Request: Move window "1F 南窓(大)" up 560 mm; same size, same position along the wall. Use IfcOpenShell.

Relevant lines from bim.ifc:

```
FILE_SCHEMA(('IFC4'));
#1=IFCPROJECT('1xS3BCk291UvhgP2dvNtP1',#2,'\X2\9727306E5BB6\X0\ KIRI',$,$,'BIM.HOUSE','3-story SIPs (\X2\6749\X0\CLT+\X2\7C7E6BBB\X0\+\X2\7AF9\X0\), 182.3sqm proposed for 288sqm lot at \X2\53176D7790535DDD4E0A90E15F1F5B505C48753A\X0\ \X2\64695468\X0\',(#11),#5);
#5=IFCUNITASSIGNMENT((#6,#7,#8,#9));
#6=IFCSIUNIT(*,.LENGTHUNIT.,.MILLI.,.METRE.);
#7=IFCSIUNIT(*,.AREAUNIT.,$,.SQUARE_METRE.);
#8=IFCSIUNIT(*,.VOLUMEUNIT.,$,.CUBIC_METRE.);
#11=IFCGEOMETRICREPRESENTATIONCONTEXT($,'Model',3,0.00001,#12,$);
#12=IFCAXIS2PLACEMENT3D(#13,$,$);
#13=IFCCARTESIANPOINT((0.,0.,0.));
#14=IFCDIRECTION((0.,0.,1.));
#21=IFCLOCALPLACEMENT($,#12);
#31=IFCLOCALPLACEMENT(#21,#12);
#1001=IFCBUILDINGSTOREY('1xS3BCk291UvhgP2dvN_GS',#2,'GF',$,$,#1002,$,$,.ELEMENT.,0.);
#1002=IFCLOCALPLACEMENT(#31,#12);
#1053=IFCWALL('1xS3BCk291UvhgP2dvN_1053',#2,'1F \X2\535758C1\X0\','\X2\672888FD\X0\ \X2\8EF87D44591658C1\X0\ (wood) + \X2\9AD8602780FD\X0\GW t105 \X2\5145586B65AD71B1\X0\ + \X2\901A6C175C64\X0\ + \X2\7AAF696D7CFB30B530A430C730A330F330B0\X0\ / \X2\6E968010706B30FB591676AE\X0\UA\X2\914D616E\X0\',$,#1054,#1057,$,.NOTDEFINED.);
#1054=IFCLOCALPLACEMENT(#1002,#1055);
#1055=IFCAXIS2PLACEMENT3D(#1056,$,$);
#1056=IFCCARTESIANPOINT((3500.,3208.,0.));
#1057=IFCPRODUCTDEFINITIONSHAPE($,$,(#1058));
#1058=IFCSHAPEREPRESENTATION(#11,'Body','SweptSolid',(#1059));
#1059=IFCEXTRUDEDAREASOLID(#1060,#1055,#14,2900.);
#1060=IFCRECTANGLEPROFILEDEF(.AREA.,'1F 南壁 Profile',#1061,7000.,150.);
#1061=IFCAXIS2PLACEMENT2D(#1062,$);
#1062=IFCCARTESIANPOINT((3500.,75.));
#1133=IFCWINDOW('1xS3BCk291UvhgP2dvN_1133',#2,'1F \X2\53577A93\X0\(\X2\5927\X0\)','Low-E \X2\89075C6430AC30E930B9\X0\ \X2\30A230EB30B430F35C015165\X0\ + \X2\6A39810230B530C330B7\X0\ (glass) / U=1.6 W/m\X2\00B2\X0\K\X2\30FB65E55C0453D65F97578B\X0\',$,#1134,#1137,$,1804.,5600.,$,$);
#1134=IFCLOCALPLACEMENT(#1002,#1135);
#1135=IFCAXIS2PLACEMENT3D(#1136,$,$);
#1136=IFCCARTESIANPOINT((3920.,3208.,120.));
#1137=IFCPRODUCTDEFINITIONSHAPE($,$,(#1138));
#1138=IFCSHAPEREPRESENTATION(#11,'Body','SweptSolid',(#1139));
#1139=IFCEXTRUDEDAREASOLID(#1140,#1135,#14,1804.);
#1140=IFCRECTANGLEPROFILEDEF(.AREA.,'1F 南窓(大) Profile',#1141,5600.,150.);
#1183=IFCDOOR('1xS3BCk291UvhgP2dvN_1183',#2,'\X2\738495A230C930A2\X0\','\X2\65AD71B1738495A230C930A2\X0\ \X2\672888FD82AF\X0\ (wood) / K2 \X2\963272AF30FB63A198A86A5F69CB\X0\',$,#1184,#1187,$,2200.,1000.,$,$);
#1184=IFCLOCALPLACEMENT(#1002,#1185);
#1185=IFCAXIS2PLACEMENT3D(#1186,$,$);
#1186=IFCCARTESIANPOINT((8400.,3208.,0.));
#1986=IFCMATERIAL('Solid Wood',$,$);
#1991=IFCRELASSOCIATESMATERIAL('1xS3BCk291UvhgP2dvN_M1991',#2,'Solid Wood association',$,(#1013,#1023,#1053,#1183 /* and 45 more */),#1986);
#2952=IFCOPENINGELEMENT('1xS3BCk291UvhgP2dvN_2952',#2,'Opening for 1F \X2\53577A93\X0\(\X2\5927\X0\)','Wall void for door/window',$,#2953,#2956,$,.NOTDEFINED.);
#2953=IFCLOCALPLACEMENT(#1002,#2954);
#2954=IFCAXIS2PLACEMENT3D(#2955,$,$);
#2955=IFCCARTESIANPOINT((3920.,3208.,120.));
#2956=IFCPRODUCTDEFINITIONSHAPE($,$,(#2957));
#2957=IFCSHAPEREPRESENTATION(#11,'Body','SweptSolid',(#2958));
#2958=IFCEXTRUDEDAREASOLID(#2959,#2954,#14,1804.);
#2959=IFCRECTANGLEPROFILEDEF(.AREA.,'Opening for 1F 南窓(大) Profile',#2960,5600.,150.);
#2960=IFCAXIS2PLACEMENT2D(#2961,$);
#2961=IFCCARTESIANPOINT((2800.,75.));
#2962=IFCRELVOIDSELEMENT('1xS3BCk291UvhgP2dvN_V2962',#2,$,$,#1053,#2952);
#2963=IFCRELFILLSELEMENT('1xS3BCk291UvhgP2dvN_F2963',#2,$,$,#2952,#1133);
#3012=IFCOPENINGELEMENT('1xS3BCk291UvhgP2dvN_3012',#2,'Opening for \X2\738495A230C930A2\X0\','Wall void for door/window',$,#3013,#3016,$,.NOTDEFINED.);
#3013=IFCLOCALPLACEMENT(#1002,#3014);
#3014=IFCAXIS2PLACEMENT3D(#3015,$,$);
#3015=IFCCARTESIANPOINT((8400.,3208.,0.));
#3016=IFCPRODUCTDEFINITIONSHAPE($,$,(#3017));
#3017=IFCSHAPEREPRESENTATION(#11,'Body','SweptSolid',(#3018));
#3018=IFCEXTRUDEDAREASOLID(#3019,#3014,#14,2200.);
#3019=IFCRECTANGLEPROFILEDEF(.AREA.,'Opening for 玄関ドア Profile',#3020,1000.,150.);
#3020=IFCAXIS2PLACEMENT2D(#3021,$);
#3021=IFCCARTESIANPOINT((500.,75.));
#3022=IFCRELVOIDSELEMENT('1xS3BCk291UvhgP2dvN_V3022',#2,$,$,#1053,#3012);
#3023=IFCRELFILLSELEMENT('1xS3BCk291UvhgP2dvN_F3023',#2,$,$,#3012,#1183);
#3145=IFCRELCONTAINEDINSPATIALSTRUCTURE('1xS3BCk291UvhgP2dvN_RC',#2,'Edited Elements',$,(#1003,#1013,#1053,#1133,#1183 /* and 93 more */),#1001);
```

```python
import numpy as np
import ifcopenshell
import ifcopenshell.api.geometry
import ifcopenshell.util.placement
import ifcopenshell.util.unit

model = ifcopenshell.open("bim.ifc")
unit_scale = ifcopenshell.util.unit.calculate_unit_scale(model)

window = model.by_guid("1xS3BCk291UvhgP2dvN_1133")
opening = window.FillsVoids[0].RelatingOpeningElement
dz = 0.56 / unit_scale

shift = np.array([0.0, 0.0, dz])
# The window is not placed relative to its opening, so move both.
for product in (opening, window):
    matrix = ifcopenshell.util.placement.get_local_placement(product.ObjectPlacement)
    matrix[:3, 3] += shift
    ifcopenshell.api.geometry.edit_object_placement(model, product=product, matrix=matrix, is_si=False)

print(f"moved by {dz * unit_scale:+.3f} m")

model.write("bim_rev.ifc")
```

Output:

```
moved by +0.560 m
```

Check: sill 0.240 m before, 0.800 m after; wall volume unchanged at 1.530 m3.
